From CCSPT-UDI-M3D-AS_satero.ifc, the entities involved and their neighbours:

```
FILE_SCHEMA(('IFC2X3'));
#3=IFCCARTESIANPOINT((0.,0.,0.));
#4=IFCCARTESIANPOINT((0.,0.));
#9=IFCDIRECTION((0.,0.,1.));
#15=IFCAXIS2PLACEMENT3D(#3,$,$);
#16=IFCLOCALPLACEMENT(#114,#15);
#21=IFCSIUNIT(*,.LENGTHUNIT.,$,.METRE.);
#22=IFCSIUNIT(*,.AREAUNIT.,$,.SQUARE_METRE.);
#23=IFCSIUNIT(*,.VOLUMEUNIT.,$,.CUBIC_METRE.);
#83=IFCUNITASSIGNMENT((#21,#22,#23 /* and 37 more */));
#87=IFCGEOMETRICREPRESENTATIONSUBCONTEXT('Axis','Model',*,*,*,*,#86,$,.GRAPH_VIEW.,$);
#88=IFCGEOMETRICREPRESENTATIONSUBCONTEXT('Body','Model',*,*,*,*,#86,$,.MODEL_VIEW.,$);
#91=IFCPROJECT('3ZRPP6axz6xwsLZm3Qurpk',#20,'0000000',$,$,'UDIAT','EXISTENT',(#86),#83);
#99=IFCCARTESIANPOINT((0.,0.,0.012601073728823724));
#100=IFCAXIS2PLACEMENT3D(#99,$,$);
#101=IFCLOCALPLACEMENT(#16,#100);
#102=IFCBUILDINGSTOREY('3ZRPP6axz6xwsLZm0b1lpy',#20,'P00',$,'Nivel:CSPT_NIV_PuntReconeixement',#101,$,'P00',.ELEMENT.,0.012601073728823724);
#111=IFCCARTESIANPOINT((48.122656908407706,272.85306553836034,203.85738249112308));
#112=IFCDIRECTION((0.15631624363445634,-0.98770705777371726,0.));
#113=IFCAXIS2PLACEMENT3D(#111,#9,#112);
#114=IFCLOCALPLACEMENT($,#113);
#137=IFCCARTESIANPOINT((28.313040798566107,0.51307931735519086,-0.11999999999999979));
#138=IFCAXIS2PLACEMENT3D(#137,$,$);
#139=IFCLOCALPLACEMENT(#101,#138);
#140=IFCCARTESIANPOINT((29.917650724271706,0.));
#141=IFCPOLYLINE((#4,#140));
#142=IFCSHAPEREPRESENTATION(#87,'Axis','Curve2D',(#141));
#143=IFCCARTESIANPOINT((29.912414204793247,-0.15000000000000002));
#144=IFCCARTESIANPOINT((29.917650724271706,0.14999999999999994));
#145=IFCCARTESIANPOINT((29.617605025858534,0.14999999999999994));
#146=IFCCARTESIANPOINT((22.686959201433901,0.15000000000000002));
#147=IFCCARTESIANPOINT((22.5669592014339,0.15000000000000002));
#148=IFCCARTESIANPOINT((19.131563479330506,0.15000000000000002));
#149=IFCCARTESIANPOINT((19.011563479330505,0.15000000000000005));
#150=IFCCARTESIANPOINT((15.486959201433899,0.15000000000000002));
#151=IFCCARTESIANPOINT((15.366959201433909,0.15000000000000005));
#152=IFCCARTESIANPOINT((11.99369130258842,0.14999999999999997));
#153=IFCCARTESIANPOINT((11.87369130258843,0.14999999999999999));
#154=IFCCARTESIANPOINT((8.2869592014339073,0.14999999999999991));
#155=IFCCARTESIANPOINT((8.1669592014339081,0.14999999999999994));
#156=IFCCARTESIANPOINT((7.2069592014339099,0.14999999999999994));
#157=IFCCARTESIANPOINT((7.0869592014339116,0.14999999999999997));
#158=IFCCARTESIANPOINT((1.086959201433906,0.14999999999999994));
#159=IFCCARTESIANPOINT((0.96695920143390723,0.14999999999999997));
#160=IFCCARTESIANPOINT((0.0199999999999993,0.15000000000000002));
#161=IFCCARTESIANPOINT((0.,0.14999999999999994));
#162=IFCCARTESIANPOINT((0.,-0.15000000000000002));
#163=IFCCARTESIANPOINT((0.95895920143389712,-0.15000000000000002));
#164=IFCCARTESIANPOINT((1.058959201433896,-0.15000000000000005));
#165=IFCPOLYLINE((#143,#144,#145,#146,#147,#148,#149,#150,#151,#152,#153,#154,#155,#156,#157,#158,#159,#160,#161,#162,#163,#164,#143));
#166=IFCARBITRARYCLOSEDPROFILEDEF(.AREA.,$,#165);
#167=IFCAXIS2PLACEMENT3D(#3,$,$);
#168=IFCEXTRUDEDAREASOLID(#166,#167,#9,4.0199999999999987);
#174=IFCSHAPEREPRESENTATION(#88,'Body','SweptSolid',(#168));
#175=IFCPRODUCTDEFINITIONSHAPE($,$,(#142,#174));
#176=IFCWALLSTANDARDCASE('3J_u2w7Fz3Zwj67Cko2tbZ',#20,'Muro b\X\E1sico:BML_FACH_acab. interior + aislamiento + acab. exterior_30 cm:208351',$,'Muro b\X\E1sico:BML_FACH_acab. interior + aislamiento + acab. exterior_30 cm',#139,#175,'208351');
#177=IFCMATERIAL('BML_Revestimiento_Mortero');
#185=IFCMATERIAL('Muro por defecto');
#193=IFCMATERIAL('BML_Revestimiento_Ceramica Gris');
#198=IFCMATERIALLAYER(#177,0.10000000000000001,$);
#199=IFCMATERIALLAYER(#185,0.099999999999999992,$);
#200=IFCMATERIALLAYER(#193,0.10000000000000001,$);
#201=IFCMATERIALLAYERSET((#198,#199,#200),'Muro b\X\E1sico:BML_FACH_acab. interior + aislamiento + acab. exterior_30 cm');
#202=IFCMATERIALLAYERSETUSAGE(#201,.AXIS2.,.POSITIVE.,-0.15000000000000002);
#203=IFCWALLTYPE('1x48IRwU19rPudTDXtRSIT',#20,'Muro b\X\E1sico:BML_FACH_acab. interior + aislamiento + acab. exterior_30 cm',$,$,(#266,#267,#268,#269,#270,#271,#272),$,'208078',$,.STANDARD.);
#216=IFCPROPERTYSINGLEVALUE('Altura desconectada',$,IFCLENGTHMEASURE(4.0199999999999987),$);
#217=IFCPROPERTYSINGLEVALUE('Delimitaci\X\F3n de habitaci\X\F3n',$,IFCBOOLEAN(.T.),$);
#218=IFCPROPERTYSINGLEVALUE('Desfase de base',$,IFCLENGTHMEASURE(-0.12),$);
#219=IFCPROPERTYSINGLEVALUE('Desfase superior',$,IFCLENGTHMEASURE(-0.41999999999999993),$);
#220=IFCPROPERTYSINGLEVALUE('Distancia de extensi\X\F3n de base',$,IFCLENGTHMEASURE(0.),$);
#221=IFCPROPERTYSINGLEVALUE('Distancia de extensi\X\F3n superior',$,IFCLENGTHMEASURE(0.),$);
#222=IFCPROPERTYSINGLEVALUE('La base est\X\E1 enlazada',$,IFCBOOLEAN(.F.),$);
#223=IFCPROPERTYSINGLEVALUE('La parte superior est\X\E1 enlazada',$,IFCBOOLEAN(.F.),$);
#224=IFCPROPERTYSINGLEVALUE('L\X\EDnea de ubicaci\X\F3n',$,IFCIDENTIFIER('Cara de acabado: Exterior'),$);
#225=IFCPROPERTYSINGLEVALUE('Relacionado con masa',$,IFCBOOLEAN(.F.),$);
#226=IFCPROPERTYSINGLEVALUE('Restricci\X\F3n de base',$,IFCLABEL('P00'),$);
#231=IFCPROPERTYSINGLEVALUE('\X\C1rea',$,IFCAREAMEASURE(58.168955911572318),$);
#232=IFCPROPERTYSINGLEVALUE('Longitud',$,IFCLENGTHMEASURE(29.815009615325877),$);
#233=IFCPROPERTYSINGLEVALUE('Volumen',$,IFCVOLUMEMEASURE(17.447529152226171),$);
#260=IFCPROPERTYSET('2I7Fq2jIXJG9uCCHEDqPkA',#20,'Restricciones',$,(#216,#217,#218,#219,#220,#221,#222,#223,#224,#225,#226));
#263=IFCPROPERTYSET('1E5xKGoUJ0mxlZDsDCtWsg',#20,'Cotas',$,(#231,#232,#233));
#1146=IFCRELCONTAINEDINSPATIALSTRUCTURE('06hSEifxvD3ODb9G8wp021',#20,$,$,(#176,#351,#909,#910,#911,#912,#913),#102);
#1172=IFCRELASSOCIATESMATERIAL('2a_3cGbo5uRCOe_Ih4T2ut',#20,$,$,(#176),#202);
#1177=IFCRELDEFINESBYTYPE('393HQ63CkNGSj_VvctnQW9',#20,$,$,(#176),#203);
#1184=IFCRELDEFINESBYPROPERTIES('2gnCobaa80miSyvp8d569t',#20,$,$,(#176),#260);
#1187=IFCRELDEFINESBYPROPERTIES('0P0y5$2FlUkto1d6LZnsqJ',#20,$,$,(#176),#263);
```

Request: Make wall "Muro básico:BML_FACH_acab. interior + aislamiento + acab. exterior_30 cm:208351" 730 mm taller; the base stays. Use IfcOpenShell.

```python
import ifcopenshell
import ifcopenshell.api.pset
import ifcopenshell.geom
import ifcopenshell.util.element
import ifcopenshell.util.representation
import ifcopenshell.util.shape
import ifcopenshell.util.unit

model = ifcopenshell.open("CCSPT-UDI-M3D-AS_satero.ifc")
unit_scale = ifcopenshell.util.unit.calculate_unit_scale(model)
area_scale = ifcopenshell.util.unit.calculate_unit_scale(model, "AREAUNIT")
volume_scale = ifcopenshell.util.unit.calculate_unit_scale(model, "VOLUMEUNIT")
settings = ifcopenshell.geom.settings()


def volume(element):
    """Net volume in cubic metres, openings subtracted."""
    shape = ifcopenshell.geom.create_shape(settings, element)
    return ifcopenshell.util.shape.get_volume(shape.geometry)


wall = model.by_guid("3J_u2w7Fz3Zwj67Cko2tbZ")
before = volume(wall)

body = ifcopenshell.util.representation.get_representation(wall, "Model", "Body")
solid = body.Items[0]
old_height = solid.Depth
solid.Depth += 0.73 / unit_scale
after = volume(wall)
thickness = 0.3  # wall thickness in metres

# Update the stored height, areas and volumes.
pset = model.by_id(ifcopenshell.util.element.get_pset(wall, "Restricciones", should_inherit=False)["id"])
ifcopenshell.api.pset.edit_pset(model, pset=pset, properties={
    "Altura desconectada": model.create_entity("IfcLengthMeasure", solid.Depth),
})
pset = model.by_id(ifcopenshell.util.element.get_pset(wall, "Cotas", should_inherit=False)["id"])
ifcopenshell.api.pset.edit_pset(model, pset=pset, properties={
    "Área": model.create_entity("IfcAreaMeasure", after / thickness / area_scale),
    "Volumen": model.create_entity("IfcVolumeMeasure", after / volume_scale),
})

print(f"height {old_height:g} -> {solid.Depth:g}, volume {before:.3f} -> {after:.3f} m3")

model.write("CCSPT-UDI-M3D-AS_satero_edited.ifc")
```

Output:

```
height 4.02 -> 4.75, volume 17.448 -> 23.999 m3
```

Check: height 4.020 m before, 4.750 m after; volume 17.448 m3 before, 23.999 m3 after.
